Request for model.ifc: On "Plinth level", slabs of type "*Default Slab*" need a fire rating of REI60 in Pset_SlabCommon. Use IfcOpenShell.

First a look at what the model holds.

```python
import ifcopenshell
import ifcopenshell.util.element

model = ifcopenshell.open("model.ifc")
print(model.schema)
storey = next(s for s in model.by_type("IfcBuildingStorey") if s.Name == "Plinth level")
slabs = [e for e in ifcopenshell.util.element.get_decomposition(storey) if e.is_a("IfcSlab")]
seen = {}
for e in slabs:
    element_type = ifcopenshell.util.element.get_type(e)
    key = (element_type.Name if element_type != e and element_type else None, ifcopenshell.util.element.get_pset(e, "Pset_SlabCommon", "FireRating"))
    seen[key] = seen.get(key, 0) + 1
for (name, value), count in sorted(seen.items(), key=str):
    print(count, "x", name, "|", value)
```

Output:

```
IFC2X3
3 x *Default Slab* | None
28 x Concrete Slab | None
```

```python
import ifcopenshell
import ifcopenshell.api.pset
import ifcopenshell.util.element

model = ifcopenshell.open("model.ifc")

storey = next(s for s in model.by_type("IfcBuildingStorey") if s.Name == "Plinth level")
slabs = [e for e in ifcopenshell.util.element.get_decomposition(storey) if e.is_a("IfcSlab")]

count = 0
for e in slabs:
    element_type = ifcopenshell.util.element.get_type(e)
    if element_type in (None, e) or element_type.Name != "*Default Slab*":
        continue
    # add_pset returns the element's existing set when there is one.
    pset = ifcopenshell.api.pset.add_pset(model, product=e, name="Pset_SlabCommon")
    ifcopenshell.api.pset.edit_pset(model, pset=pset, properties={"FireRating": "REI60"})
    count += 1

print(count, "slabs updated")

model.write("model-out.ifc")
```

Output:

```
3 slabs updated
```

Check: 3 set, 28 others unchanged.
